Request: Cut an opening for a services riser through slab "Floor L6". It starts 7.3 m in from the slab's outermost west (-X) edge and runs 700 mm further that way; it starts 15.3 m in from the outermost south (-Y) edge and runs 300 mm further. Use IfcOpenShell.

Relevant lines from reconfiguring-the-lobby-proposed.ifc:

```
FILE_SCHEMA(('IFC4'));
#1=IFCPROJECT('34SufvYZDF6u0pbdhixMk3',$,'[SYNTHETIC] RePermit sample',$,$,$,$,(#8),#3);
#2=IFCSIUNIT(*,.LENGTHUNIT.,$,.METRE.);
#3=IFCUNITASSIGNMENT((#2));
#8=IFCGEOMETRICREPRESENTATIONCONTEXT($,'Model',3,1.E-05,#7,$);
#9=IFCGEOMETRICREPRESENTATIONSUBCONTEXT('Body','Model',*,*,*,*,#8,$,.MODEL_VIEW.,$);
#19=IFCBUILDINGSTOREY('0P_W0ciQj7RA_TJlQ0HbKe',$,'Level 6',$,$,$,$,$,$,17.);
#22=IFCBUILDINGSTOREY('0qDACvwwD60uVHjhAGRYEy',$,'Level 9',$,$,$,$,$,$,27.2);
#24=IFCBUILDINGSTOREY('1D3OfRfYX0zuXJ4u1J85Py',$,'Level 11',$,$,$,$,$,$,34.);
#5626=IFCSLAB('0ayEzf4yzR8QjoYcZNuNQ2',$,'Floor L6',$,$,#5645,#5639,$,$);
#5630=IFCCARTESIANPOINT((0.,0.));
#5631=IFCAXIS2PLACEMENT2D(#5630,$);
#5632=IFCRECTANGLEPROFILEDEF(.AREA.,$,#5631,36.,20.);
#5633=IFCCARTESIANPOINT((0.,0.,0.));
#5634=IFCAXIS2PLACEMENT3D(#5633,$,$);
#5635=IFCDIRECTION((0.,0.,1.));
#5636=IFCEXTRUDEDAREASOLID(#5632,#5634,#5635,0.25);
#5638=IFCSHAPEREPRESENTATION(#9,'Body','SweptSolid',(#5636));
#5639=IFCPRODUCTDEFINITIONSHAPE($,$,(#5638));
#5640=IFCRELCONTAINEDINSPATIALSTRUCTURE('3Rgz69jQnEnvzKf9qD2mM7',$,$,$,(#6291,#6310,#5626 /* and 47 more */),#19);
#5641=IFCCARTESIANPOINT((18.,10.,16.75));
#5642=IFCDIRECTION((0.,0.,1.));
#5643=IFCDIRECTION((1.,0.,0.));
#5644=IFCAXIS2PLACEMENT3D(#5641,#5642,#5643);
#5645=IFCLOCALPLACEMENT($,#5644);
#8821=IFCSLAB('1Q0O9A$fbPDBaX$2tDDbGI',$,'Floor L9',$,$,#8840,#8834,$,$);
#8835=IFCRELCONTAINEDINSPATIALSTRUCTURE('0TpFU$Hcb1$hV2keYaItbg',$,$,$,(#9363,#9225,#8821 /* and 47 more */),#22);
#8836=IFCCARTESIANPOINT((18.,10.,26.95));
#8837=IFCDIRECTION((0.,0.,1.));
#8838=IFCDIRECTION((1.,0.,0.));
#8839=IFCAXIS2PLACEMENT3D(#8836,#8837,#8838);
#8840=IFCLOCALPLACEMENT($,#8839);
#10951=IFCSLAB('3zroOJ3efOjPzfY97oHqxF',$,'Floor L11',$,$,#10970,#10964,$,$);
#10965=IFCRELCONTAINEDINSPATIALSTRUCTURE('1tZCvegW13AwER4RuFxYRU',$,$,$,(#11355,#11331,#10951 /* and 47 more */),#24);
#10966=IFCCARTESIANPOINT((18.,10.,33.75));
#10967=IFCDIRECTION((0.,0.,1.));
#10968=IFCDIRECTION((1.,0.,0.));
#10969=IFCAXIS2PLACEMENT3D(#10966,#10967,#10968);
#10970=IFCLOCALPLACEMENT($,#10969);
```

```python
import numpy as np
import ifcopenshell
import ifcopenshell.api.feature
import ifcopenshell.api.geometry
import ifcopenshell.api.root
import ifcopenshell.geom
import ifcopenshell.util.placement
import ifcopenshell.util.representation
import ifcopenshell.util.shape
import ifcopenshell.util.unit

model = ifcopenshell.open("reconfiguring-the-lobby-proposed.ifc")
unit_scale = ifcopenshell.util.unit.calculate_unit_scale(model)
settings = ifcopenshell.geom.settings()


def volume(element):
    """Net volume in cubic metres, openings subtracted."""
    shape = ifcopenshell.geom.create_shape(settings, element)
    return ifcopenshell.util.shape.get_volume(shape.geometry)


slab = model.by_guid("0ayEzf4yzR8QjoYcZNuNQ2")
before = volume(slab)

# Extent in the slab's own axes, in metres. The edges named are its -X and -Y sides.
slab_shape = ifcopenshell.geom.create_shape(settings, slab)
vertices = ifcopenshell.util.shape.get_vertices(slab_shape.geometry)
x_min, y_min, bottom = vertices.min(axis=0)
top = vertices[:, 2].max()

opening = ifcopenshell.api.root.create_entity(model, ifc_class="IfcOpeningElement", name="Services riser opening", predefined_type="OPENING")
context = ifcopenshell.util.representation.get_context(model, "Model", "Body", "MODEL_VIEW")
width, depth = 0.7, 0.3
outline = [(0.0, 0.0), (width, 0.0), (width, depth), (0.0, depth), (0.0, 0.0)]
# Overshoot both faces by 50 mm so the cut is clean.
shape = ifcopenshell.api.geometry.add_slab_representation(
    model, context=context, depth=top - bottom + 0.1, polyline=outline
)
ifcopenshell.api.geometry.assign_representation(model, product=opening, representation=shape)

matrix = ifcopenshell.util.placement.get_local_placement(slab.ObjectPlacement)
matrix[:, 3] = matrix @ np.append(np.array([x_min + 7.3, y_min + 15.3, bottom - 0.05]) / unit_scale, 1.0)
ifcopenshell.api.geometry.edit_object_placement(model, product=opening, matrix=matrix, is_si=False)
ifcopenshell.api.feature.add_feature(model, feature=opening, element=slab)

after = volume(slab)

print(f"slab volume {before:.3f} -> {after:.3f} m3")

model.write("reconfiguring-the-lobby-proposed_edited.ifc")
```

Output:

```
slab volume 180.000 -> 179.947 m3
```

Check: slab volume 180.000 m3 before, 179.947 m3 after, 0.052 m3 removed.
